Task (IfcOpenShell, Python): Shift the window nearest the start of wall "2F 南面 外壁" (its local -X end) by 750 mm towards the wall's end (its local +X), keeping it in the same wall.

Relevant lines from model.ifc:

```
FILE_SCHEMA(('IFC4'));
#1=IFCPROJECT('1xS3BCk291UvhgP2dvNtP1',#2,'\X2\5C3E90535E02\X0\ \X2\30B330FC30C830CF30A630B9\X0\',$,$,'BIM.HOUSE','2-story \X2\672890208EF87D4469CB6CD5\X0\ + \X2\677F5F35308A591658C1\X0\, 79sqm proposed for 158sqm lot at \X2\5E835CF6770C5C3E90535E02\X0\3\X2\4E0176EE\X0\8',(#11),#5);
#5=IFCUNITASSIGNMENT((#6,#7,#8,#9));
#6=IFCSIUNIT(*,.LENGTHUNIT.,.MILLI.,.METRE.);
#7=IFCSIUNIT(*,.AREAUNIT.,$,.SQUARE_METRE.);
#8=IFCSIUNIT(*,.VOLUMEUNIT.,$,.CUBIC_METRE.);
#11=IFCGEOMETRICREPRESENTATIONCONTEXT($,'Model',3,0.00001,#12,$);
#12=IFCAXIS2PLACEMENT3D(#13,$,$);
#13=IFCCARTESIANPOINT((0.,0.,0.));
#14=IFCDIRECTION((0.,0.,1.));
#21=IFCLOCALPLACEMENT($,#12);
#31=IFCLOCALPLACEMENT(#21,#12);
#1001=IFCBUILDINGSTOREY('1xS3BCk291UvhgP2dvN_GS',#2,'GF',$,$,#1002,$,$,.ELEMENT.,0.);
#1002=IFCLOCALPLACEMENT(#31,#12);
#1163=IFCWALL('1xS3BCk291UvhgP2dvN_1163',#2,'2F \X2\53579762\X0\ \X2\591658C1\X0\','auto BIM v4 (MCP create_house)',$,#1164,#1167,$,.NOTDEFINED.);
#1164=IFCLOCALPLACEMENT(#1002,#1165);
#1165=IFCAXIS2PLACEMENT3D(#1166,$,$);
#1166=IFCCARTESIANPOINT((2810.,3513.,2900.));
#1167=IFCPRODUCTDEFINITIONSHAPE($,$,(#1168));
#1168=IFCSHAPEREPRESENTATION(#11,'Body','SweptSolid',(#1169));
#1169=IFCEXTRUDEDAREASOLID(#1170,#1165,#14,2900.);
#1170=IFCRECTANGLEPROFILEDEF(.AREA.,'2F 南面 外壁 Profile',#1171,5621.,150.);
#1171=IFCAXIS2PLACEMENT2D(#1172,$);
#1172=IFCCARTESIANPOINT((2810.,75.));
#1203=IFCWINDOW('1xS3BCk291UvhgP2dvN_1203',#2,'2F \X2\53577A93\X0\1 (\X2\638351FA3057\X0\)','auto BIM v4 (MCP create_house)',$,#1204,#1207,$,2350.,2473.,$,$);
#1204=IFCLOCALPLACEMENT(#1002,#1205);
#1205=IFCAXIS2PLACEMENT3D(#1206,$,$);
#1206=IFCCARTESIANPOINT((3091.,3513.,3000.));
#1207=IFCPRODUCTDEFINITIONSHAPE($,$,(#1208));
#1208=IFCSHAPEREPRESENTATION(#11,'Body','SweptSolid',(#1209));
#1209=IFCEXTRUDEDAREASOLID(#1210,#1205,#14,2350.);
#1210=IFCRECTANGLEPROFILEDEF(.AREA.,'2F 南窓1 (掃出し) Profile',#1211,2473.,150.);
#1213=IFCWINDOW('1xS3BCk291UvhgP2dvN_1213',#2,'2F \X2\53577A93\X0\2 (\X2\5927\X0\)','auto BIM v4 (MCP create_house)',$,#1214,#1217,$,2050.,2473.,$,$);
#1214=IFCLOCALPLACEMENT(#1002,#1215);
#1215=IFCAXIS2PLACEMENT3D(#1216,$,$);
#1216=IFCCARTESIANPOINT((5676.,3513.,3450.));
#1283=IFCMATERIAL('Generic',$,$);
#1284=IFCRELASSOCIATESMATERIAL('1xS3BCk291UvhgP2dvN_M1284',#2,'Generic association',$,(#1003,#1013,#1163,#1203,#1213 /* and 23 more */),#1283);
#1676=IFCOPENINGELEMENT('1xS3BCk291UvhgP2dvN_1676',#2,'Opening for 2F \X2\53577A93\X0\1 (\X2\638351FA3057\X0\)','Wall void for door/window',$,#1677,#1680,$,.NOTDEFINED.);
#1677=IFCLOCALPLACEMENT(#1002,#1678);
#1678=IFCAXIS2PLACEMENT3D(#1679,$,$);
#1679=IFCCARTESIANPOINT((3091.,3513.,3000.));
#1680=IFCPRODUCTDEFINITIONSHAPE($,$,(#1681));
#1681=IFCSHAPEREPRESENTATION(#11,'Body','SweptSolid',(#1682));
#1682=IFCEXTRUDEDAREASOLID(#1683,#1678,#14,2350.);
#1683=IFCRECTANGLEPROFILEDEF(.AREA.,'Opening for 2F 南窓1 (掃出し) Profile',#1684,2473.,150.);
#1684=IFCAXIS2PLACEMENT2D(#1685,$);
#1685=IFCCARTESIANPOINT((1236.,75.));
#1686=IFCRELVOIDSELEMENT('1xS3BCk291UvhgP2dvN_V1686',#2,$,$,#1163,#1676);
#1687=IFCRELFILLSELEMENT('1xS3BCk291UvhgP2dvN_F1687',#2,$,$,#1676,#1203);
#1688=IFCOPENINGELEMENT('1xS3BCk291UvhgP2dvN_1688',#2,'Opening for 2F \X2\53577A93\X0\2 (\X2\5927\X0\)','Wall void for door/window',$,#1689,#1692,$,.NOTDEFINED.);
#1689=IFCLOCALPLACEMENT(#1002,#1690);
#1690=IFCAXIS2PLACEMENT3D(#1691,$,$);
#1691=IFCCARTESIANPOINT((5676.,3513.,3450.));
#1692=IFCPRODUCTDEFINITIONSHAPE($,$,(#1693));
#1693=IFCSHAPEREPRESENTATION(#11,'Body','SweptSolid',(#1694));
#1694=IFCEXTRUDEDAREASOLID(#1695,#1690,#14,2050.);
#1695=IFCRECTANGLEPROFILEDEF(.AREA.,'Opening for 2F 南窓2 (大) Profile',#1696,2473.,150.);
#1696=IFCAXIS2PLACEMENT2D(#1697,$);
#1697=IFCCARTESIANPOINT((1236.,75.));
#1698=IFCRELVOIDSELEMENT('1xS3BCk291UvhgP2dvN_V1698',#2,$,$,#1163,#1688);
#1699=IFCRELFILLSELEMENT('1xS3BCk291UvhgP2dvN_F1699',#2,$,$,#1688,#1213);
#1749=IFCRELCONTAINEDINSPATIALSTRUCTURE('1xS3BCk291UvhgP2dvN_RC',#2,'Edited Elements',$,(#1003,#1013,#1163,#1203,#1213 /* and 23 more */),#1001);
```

```python
import ifcopenshell
import ifcopenshell.api.geometry
import ifcopenshell.util.placement
import ifcopenshell.util.unit

model = ifcopenshell.open("model.ifc")
unit_scale = ifcopenshell.util.unit.calculate_unit_scale(model)

window = model.by_id(1203)
opening = window.FillsVoids[0].RelatingOpeningElement
wall = opening.VoidsElements[0].RelatingBuildingElement

wall_matrix = ifcopenshell.util.placement.get_local_placement(wall.ObjectPlacement)
shift = wall_matrix[:3, 0] * 0.75 / unit_scale
before = ifcopenshell.util.placement.get_local_placement(window.ObjectPlacement)[:3, 3].copy()

# The window is not placed relative to its opening, so move both.
for product in (opening, window):
    matrix = ifcopenshell.util.placement.get_local_placement(product.ObjectPlacement)
    matrix[:3, 3] += shift
    ifcopenshell.api.geometry.edit_object_placement(model, product=product, matrix=matrix, is_si=False)

after = ifcopenshell.util.placement.get_local_placement(window.ObjectPlacement)[:3, 3]
print("window moved by", (after - before).round(3) + 0.0)

model.write("model_v2.ifc")
```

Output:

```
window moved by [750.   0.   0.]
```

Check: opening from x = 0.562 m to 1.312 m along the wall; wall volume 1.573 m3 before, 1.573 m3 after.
